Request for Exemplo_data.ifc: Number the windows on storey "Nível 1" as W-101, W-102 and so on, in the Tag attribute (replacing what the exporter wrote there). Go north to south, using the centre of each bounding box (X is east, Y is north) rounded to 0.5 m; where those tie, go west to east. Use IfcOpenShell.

First a look at what the model holds.

```python
import ifcopenshell
import ifcopenshell.util.element
import ifcopenshell.util.placement

model = ifcopenshell.open("Exemplo_data.ifc")
print(model.schema)
storey = next(s for s in model.by_type("IfcBuildingStorey") if s.Name == "Nível 1")
windows = [e for e in ifcopenshell.util.element.get_decomposition(storey) if e.is_a("IfcWindow")]
for e in sorted(windows, key=lambda e: e.id()):
    origin = ifcopenshell.util.placement.get_local_placement(e.ObjectPlacement)[:3, 3]
    print(e.id(), e.Tag, e.Name, origin.round(2) + 0.0, sep=" | ")
```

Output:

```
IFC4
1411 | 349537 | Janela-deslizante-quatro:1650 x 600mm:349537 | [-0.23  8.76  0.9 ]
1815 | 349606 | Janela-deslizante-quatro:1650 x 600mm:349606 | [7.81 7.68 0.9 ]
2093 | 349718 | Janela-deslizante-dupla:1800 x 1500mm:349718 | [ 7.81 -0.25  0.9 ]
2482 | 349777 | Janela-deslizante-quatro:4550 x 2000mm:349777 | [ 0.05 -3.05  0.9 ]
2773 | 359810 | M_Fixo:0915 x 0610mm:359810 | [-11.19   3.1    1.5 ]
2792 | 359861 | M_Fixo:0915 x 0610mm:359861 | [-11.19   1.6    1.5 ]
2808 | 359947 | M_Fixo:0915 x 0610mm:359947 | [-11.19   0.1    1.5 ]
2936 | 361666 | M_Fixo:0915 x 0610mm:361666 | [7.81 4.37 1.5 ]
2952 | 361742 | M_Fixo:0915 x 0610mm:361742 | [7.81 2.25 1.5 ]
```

```python
import ifcopenshell
import ifcopenshell.geom
import ifcopenshell.util.element
import ifcopenshell.util.shape

model = ifcopenshell.open("Exemplo_data.ifc")
settings = ifcopenshell.geom.settings()
settings.set("use-world-coords", True)


def centre(element):
    shape = ifcopenshell.geom.create_shape(settings, element)
    return ifcopenshell.util.shape.get_bbox_centroid(shape.geometry)


storey = next(s for s in model.by_type("IfcBuildingStorey") if s.Name == "Nível 1")
windows = [e for e in ifcopenshell.util.element.get_decomposition(storey) if e.is_a("IfcWindow")]

# Insertion points can sit at a corner or the storey origin, so sort by the geometry (in metres).
centres = {e: centre(e) for e in windows}
windows.sort(key=lambda e: (-round(centres[e][1] / 0.5), centres[e][0]))

for i, e in enumerate(windows, start=1):
    number = f"W-1{i:02d}"
    e.Tag = number
    print(e.id(), number)

model.write("Exemplo_data_edited.ifc")
```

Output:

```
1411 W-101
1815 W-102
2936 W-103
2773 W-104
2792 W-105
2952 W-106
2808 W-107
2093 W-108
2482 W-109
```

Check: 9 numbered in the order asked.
